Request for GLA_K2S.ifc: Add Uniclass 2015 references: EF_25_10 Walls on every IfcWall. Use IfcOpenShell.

First a look at what the model holds.

```python
import ifcopenshell

model = ifcopenshell.open("GLA_K2S.ifc")
print(model.schema)
print("classifications:", [c.Name for c in model.by_type("IfcClassification")])
for ifc_class in ("IfcDoor", "IfcRoof", "IfcStair", "IfcWall", "IfcWindow"):
    print(ifc_class, len(model.by_type(ifc_class)))
```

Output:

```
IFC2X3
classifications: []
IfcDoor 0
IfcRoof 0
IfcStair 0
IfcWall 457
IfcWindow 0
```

```python
import ifcopenshell
import ifcopenshell.api.classification

model = ifcopenshell.open("GLA_K2S.ifc")

# IFC2X3 requires Source and Edition and has no link from the project to the system.
system = model.create_entity("IfcClassification", Source="NBS", Edition="2015", Name="Uniclass 2015")

codes = {
    "IfcWall": ("EF_25_10", "Walls"),
}
for ifc_class, (code, name) in codes.items():
    products = model.by_type(ifc_class)
    ifcopenshell.api.classification.add_reference(
        model, products=products, classification=system, identification=code, name=name
    )
    print(code, len(products))

model.write("GLA_K2S_rev.ifc")
```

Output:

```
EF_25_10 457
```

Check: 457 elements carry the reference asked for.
